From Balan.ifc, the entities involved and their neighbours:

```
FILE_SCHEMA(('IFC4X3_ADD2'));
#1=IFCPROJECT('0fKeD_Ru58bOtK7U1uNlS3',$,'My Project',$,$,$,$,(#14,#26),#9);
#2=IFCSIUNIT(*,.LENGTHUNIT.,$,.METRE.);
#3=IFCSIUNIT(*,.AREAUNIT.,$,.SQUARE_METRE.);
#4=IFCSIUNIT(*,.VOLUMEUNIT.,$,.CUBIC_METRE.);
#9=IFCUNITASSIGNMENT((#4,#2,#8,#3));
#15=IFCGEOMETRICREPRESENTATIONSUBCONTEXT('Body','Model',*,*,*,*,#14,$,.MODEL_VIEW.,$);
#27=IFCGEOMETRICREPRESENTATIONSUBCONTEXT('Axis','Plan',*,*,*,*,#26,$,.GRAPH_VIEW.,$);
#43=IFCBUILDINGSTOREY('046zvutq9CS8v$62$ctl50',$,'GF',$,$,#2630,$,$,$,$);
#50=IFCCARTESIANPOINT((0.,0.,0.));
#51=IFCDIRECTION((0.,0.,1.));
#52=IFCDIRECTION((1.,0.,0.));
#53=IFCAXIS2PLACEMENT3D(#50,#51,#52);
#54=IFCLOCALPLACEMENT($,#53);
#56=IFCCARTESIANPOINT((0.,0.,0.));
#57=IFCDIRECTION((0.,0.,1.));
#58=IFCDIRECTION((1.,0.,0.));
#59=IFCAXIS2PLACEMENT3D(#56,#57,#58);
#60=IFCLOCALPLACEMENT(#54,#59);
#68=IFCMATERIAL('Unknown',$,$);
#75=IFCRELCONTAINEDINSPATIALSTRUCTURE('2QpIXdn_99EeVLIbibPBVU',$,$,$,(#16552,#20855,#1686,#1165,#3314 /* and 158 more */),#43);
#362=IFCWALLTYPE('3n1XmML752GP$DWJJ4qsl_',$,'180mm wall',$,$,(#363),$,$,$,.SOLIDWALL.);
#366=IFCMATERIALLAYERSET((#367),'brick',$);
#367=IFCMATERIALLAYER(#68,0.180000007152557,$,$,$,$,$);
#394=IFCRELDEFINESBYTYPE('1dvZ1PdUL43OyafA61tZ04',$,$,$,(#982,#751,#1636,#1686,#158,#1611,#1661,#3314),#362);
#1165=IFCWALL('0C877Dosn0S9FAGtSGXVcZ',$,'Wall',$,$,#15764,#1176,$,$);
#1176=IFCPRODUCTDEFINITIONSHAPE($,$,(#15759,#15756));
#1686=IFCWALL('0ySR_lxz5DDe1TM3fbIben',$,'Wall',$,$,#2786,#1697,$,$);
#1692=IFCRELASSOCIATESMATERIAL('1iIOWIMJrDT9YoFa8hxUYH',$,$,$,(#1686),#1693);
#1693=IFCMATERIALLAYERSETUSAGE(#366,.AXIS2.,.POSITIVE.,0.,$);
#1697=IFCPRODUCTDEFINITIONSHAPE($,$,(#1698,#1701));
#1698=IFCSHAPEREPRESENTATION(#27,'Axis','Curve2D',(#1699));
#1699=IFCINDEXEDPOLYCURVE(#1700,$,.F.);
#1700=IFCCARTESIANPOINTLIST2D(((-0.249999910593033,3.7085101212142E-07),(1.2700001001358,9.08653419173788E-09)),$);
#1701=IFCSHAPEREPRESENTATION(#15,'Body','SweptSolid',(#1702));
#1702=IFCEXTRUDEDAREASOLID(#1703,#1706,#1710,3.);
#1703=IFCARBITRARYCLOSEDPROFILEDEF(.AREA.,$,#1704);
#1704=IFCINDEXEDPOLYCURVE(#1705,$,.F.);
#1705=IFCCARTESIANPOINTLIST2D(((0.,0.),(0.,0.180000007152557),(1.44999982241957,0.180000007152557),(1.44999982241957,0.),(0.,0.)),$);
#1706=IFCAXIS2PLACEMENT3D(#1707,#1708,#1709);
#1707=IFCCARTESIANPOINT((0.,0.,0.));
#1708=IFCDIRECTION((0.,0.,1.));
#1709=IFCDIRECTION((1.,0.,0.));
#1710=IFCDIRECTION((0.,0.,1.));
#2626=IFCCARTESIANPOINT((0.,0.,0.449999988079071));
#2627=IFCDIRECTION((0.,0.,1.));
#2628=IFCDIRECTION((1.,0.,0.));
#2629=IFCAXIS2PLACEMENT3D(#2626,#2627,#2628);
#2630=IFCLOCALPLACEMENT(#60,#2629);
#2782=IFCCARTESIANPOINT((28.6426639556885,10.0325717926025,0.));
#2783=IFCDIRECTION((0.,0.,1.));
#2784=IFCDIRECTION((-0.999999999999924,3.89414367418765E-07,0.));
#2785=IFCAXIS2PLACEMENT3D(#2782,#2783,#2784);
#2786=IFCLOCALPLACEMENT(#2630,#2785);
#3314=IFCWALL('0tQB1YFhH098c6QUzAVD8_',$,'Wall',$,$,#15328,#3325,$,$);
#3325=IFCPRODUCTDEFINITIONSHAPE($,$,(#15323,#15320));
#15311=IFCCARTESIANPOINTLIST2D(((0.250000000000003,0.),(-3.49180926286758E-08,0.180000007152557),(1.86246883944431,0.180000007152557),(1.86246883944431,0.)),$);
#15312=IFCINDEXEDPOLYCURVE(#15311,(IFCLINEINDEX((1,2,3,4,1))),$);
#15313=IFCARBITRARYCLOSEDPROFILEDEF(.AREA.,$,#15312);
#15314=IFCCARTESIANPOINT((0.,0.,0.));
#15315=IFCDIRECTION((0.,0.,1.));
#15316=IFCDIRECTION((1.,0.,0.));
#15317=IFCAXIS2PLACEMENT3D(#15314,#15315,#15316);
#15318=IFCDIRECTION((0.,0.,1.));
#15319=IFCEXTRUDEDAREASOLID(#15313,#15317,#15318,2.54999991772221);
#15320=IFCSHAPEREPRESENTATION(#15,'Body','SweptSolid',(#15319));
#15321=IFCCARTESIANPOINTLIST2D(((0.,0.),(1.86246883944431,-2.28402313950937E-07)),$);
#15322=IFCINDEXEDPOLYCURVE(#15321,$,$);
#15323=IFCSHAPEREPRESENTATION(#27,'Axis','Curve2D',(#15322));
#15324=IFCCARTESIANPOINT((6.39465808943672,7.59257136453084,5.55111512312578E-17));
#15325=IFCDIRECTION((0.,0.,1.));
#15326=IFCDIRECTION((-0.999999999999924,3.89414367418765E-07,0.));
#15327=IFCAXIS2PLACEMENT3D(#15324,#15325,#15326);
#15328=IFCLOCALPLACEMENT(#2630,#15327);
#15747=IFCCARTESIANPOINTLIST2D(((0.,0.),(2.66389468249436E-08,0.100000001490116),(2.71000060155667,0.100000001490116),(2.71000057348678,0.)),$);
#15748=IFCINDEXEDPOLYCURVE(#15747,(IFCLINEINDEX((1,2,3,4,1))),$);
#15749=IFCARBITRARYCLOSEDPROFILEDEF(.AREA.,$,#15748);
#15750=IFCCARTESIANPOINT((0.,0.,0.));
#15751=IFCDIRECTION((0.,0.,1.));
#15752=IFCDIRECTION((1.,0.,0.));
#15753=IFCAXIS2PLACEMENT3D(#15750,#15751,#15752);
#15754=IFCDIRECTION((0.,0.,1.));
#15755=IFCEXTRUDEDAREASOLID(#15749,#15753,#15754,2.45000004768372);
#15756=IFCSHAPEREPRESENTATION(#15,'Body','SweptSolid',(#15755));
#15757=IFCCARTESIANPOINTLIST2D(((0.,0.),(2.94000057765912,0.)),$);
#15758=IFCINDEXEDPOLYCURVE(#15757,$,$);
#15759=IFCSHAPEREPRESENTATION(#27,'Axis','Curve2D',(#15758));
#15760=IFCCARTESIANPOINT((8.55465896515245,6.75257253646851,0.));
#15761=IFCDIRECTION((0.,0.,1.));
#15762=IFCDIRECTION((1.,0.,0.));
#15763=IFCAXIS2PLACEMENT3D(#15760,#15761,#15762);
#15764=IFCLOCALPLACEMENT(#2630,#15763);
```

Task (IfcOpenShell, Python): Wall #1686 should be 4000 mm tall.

```python
import ifcopenshell
import ifcopenshell.geom
import ifcopenshell.util.representation
import ifcopenshell.util.shape

model = ifcopenshell.open("Balan.ifc")
settings = ifcopenshell.geom.settings()


def volume(element):
    """Net volume in cubic metres, openings subtracted."""
    shape = ifcopenshell.geom.create_shape(settings, element)
    return ifcopenshell.util.shape.get_volume(shape.geometry)


wall = model.by_guid("0ySR_lxz5DDe1TM3fbIben")
before = volume(wall)

body = ifcopenshell.util.representation.get_representation(wall, "Model", "Body")
solid = body.Items[0]
old_height = solid.Depth
solid.Depth = 4.0
after = volume(wall)

print(f"height {old_height:g} -> {solid.Depth:g}, volume {before:.3f} -> {after:.3f} m3")

model.write("Balan_updated.ifc")
```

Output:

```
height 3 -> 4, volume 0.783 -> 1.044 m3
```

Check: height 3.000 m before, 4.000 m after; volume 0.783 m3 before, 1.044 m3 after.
